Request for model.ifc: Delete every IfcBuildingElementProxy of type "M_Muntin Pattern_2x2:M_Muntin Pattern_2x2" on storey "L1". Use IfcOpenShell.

First a look at what the model holds.

```python
import ifcopenshell
import ifcopenshell.util.element

model = ifcopenshell.open("model.ifc")
print(model.schema)
storey = next(s for s in model.by_type("IfcBuildingStorey") if s.Name == "L1")
proxies = [e for e in ifcopenshell.util.element.get_decomposition(storey) if e.is_a("IfcBuildingElementProxy")]
seen = {}
for e in proxies:
    element_type = ifcopenshell.util.element.get_type(e)
    name = element_type.Name if element_type not in (None, e) else None
    seen[name] = seen.get(name, 0) + 1
for name, count in sorted(seen.items(), key=str):
    print(count, "x", name)
```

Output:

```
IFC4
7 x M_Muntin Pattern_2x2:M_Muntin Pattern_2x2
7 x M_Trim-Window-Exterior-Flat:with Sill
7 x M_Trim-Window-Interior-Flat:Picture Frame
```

```python
import ifcopenshell
import ifcopenshell.api.root
import ifcopenshell.util.element

model = ifcopenshell.open("model.ifc")

storey = next(s for s in model.by_type("IfcBuildingStorey") if s.Name == "L1")
proxies = [e for e in ifcopenshell.util.element.get_decomposition(storey) if e.is_a("IfcBuildingElementProxy")]
targets = [e for e in proxies if (t := ifcopenshell.util.element.get_type(e)) not in (None, e) and t.Name == "M_Muntin Pattern_2x2:M_Muntin Pattern_2x2"]

for e in targets:
    ifcopenshell.api.root.remove_product(model, product=e)
print(len(targets), "removed")

model.write("model_v2.ifc")
```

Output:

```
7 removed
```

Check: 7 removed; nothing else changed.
